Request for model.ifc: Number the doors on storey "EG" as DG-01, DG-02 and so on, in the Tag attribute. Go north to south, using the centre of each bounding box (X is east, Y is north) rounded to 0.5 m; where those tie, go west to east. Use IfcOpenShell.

First a look at what the model holds.

```python
import ifcopenshell
import ifcopenshell.util.element
import ifcopenshell.util.placement

model = ifcopenshell.open("model.ifc")
print(model.schema)
storey = next(s for s in model.by_type("IfcBuildingStorey") if s.Name == "EG")
doors = [e for e in ifcopenshell.util.element.get_decomposition(storey) if e.is_a("IfcDoor")]
for e in sorted(doors, key=lambda e: e.id()):
    origin = ifcopenshell.util.placement.get_local_placement(e.ObjectPlacement)[:3, 3]
    print(e.id(), e.Tag, e.Name, origin.round(2) + 0.0, sep=" | ")
```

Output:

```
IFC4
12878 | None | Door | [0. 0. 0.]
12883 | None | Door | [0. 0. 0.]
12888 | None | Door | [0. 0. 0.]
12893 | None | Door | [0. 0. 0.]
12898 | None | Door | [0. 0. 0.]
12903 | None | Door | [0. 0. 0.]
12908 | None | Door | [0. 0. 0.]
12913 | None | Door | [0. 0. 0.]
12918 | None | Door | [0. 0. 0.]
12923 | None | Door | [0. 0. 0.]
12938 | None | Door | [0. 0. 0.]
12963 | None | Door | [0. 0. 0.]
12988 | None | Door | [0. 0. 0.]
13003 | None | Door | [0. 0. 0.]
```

```python
import ifcopenshell
import ifcopenshell.geom
import ifcopenshell.util.element
import ifcopenshell.util.shape

model = ifcopenshell.open("model.ifc")
settings = ifcopenshell.geom.settings()
settings.set("use-world-coords", True)


def centre(element):
    shape = ifcopenshell.geom.create_shape(settings, element)
    return ifcopenshell.util.shape.get_bbox_centroid(shape.geometry)


storey = next(s for s in model.by_type("IfcBuildingStorey") if s.Name == "EG")
doors = [e for e in ifcopenshell.util.element.get_decomposition(storey) if e.is_a("IfcDoor")]

# Insertion points can sit at a corner or the storey origin, so sort by the geometry (in metres).
centres = {e: centre(e) for e in doors}
doors.sort(key=lambda e: (-round(centres[e][1] / 0.5), centres[e][0]))

for i, e in enumerate(doors, start=1):
    number = f"DG-{i:02d}"
    e.Tag = number
    print(e.id(), number)

model.write("model_rev.ifc")
```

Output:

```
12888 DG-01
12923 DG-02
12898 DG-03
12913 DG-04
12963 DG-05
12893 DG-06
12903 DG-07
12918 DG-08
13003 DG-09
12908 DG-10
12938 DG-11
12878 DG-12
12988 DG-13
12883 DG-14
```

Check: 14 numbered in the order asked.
